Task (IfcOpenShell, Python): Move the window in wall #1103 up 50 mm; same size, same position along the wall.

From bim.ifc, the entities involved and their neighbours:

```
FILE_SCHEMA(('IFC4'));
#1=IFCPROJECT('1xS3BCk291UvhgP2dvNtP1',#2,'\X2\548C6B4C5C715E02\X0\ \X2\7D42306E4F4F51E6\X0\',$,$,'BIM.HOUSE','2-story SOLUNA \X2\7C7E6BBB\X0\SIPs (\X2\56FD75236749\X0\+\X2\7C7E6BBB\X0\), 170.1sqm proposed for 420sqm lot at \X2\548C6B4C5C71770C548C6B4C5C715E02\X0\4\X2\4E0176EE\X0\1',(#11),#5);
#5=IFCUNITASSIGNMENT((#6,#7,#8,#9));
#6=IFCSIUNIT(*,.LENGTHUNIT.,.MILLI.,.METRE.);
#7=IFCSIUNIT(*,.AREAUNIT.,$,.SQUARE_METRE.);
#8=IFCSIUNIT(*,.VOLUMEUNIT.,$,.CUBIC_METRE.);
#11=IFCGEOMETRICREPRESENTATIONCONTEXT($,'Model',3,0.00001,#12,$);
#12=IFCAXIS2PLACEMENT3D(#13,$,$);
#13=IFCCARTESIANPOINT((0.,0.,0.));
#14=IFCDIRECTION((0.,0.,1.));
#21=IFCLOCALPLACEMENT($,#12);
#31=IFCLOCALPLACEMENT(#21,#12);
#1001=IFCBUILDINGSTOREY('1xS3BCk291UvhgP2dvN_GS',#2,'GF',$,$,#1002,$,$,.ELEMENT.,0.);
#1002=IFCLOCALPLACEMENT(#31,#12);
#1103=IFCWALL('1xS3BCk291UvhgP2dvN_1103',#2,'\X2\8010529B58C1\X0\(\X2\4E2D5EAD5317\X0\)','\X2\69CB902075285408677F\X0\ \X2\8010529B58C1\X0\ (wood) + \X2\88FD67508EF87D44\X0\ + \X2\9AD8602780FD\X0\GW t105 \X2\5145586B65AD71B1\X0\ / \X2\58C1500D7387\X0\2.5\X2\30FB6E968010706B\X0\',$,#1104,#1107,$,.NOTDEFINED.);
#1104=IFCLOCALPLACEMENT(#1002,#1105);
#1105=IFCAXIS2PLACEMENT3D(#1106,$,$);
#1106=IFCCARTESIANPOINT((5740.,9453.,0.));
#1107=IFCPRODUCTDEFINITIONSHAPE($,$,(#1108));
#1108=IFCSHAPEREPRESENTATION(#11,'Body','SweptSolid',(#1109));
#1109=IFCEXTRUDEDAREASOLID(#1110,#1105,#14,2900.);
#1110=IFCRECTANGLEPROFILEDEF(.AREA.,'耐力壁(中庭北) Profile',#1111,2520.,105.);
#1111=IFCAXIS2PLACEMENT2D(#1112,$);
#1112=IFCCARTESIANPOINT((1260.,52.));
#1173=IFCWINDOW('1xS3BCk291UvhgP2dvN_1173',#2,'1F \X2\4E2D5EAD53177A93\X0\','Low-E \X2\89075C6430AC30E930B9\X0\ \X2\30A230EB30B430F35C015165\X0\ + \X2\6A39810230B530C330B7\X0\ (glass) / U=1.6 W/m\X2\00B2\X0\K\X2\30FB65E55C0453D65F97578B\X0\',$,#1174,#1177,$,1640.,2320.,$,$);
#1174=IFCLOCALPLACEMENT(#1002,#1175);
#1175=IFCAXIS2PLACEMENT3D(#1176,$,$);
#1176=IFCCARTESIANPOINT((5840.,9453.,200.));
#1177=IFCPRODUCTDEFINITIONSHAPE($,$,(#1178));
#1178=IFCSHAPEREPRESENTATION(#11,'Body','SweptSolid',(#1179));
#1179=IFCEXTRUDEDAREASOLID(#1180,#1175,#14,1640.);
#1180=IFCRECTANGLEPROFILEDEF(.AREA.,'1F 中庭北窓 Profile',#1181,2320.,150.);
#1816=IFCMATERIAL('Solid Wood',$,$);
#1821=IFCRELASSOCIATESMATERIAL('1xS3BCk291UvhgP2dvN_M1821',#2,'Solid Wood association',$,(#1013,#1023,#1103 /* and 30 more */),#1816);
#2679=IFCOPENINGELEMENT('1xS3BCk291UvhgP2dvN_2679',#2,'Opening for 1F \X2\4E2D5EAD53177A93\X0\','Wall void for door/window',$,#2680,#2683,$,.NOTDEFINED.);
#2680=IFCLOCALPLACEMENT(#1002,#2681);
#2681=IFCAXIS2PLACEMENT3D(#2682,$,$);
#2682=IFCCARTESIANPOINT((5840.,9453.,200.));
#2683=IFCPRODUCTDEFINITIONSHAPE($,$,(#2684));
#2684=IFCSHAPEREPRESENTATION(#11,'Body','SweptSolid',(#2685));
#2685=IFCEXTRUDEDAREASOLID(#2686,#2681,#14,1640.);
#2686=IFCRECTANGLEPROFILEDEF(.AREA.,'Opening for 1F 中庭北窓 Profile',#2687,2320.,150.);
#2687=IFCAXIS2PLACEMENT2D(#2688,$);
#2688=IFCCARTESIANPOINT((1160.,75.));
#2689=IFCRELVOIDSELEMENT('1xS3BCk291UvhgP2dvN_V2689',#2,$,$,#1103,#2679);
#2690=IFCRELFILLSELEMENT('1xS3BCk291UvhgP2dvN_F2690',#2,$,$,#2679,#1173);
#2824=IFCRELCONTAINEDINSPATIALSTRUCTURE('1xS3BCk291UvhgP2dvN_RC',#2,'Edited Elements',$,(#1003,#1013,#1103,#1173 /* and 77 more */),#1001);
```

```python
import numpy as np
import ifcopenshell
import ifcopenshell.api.geometry
import ifcopenshell.util.placement
import ifcopenshell.util.unit

model = ifcopenshell.open("bim.ifc")
unit_scale = ifcopenshell.util.unit.calculate_unit_scale(model)

window = model.by_guid("1xS3BCk291UvhgP2dvN_1173")
opening = window.FillsVoids[0].RelatingOpeningElement
dz = 0.05 / unit_scale

shift = np.array([0.0, 0.0, dz])
# The window is not placed relative to its opening, so move both.
for product in (opening, window):
    matrix = ifcopenshell.util.placement.get_local_placement(product.ObjectPlacement)
    matrix[:3, 3] += shift
    ifcopenshell.api.geometry.edit_object_placement(model, product=product, matrix=matrix, is_si=False)

print(f"moved by {dz * unit_scale:+.3f} m")

model.write("bim-out.ifc")
```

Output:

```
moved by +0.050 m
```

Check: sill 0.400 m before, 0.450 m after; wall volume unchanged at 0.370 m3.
